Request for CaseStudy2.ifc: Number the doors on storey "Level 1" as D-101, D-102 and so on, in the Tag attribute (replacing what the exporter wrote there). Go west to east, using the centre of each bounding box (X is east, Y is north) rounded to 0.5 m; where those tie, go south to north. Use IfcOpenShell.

First a look at what the model holds.

```python
import ifcopenshell
import ifcopenshell.util.element
import ifcopenshell.util.placement

model = ifcopenshell.open("CaseStudy2.ifc")
print(model.schema)
storey = next(s for s in model.by_type("IfcBuildingStorey") if s.Name == "Level 1")
doors = [e for e in ifcopenshell.util.element.get_decomposition(storey) if e.is_a("IfcDoor")]
for e in sorted(doors, key=lambda e: e.id()):
    origin = ifcopenshell.util.placement.get_local_placement(e.ObjectPlacement)[:3, 3]
    print(e.id(), e.Tag, e.Name, origin.round(2) + 0.0, sep=" | ")
```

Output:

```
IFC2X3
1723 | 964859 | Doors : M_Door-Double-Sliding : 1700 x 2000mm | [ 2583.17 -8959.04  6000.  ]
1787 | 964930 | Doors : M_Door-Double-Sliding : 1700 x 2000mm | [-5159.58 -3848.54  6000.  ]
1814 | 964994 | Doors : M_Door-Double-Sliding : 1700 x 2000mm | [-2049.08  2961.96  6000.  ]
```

```python
import ifcopenshell
import ifcopenshell.geom
import ifcopenshell.util.element
import ifcopenshell.util.shape

model = ifcopenshell.open("CaseStudy2.ifc")
settings = ifcopenshell.geom.settings()
settings.set("use-world-coords", True)


def centre(element):
    shape = ifcopenshell.geom.create_shape(settings, element)
    return ifcopenshell.util.shape.get_bbox_centroid(shape.geometry)


storey = next(s for s in model.by_type("IfcBuildingStorey") if s.Name == "Level 1")
doors = [e for e in ifcopenshell.util.element.get_decomposition(storey) if e.is_a("IfcDoor")]

# Insertion points can sit at a corner or the storey origin, so sort by the geometry (in metres).
centres = {e: centre(e) for e in doors}
doors.sort(key=lambda e: (round(centres[e][0] / 0.5), centres[e][1]))

for i, e in enumerate(doors, start=1):
    number = f"D-1{i:02d}"
    e.Tag = number
    print(e.id(), number)

model.write("CaseStudy2-out.ifc")
```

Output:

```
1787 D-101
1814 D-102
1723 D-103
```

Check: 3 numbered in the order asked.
